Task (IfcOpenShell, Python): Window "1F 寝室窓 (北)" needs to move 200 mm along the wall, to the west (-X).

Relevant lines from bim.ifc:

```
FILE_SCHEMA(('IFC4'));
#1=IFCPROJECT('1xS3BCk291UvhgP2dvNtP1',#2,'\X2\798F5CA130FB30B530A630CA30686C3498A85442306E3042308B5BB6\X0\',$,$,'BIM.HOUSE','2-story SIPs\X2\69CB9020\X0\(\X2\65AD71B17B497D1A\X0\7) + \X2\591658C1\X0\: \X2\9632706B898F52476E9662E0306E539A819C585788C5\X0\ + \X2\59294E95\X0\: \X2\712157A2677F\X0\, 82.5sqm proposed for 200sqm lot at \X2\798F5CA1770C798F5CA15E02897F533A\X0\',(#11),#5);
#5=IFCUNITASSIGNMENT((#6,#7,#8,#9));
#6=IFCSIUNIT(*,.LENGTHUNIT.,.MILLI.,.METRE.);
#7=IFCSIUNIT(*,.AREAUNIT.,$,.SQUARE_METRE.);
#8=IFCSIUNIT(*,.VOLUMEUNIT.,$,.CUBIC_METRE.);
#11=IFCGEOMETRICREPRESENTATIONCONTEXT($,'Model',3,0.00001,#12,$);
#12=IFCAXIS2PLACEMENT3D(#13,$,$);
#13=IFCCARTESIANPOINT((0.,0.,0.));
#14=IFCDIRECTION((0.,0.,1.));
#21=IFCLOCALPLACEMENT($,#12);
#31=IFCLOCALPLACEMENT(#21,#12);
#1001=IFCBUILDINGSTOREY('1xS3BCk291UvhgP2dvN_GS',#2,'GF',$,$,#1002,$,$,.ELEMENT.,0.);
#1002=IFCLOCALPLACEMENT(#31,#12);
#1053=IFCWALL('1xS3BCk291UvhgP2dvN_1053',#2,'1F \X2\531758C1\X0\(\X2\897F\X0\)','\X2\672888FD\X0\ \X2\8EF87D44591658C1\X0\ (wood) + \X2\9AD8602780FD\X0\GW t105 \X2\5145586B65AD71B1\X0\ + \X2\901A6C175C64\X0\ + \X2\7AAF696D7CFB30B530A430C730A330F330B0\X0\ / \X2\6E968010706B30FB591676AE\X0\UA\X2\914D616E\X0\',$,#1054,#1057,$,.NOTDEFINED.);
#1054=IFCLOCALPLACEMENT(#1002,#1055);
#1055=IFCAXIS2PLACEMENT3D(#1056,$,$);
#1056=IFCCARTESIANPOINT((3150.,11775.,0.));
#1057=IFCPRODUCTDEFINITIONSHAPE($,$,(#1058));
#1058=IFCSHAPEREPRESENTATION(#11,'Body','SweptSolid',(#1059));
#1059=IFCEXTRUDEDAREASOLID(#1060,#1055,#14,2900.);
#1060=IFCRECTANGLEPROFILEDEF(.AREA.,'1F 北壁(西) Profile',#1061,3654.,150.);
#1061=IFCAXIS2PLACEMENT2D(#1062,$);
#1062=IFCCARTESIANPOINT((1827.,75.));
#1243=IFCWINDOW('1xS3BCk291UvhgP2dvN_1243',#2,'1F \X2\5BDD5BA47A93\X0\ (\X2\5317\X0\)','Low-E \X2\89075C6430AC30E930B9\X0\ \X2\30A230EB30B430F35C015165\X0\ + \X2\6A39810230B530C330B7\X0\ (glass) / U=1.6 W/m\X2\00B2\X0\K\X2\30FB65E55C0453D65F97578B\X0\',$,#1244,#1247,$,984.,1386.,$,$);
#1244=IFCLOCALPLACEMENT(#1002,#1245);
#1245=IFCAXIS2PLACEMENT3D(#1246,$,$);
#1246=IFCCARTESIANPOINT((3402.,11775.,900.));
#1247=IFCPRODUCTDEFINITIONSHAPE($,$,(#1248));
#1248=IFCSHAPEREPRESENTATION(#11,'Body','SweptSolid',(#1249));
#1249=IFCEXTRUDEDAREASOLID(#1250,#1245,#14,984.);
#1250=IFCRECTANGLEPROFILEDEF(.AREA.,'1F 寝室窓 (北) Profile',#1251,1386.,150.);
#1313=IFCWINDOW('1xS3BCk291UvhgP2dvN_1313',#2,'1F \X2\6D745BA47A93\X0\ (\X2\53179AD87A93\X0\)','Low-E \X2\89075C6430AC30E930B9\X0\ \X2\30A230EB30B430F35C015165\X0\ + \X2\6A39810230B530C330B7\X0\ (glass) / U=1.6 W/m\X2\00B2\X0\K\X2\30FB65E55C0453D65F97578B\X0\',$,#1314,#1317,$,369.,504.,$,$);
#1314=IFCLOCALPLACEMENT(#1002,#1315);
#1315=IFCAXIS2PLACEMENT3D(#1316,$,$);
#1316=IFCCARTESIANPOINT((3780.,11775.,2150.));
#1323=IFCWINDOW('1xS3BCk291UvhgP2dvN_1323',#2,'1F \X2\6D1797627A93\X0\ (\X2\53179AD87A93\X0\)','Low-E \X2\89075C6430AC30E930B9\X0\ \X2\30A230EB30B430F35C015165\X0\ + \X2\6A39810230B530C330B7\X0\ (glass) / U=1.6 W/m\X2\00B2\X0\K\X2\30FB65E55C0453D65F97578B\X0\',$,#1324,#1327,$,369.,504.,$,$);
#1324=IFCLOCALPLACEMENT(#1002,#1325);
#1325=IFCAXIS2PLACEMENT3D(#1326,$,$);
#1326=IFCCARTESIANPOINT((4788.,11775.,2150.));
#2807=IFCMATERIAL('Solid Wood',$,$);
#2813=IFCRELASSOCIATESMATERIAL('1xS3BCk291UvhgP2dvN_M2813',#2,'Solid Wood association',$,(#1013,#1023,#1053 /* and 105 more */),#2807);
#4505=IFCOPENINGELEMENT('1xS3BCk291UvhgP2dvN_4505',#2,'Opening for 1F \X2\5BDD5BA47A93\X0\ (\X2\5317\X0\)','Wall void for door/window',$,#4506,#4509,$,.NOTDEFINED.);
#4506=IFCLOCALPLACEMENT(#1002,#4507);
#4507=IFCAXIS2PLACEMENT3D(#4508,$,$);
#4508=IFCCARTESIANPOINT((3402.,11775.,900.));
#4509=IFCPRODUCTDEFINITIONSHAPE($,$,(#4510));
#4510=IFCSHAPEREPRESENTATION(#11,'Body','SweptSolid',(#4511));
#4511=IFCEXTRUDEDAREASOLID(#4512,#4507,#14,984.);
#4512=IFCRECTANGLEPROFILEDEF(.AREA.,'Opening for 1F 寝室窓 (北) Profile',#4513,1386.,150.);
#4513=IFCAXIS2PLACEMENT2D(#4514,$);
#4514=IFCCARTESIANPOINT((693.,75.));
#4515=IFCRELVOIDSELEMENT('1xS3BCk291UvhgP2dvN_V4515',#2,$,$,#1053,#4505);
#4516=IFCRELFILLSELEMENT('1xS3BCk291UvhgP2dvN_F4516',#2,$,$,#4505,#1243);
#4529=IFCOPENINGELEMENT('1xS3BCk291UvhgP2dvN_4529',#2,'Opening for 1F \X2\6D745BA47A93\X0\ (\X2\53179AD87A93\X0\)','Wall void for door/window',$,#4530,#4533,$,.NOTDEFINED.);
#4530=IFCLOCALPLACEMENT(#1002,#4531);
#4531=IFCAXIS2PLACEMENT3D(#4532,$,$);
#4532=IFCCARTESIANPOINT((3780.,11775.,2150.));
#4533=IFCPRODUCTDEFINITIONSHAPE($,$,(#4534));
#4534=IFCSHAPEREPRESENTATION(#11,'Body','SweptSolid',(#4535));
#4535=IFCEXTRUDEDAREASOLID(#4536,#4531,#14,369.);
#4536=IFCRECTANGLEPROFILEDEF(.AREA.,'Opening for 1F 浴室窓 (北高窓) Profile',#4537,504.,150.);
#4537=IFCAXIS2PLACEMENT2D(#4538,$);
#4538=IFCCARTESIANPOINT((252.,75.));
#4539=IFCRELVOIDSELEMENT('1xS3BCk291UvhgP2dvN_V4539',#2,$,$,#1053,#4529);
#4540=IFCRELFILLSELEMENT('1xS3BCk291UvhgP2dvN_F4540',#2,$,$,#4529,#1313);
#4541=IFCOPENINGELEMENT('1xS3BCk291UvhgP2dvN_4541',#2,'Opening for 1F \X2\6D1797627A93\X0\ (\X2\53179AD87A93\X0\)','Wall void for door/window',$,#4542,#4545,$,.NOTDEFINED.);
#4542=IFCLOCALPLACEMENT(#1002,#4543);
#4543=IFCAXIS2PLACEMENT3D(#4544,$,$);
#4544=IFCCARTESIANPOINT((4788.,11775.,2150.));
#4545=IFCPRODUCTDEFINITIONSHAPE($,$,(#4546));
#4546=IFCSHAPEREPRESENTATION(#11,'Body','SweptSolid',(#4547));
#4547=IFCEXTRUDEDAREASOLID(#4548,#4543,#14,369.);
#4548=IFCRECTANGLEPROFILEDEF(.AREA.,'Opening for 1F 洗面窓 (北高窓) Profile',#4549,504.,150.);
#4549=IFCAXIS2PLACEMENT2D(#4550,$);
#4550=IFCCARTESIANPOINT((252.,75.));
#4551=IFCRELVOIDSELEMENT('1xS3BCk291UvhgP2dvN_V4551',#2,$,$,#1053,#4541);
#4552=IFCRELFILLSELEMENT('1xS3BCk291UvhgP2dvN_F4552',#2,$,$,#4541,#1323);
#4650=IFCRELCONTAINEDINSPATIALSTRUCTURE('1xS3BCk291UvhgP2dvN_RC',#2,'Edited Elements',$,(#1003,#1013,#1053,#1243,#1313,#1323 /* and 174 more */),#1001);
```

```python
import ifcopenshell
import ifcopenshell.api.geometry
import ifcopenshell.util.placement

model = ifcopenshell.open("bim.ifc")

window = model.by_guid("1xS3BCk291UvhgP2dvN_1243")
opening = window.FillsVoids[0].RelatingOpeningElement
wall = opening.VoidsElements[0].RelatingBuildingElement

wall_matrix = ifcopenshell.util.placement.get_local_placement(wall.ObjectPlacement)
shift = wall_matrix[:3, 0] * -200.0
before = ifcopenshell.util.placement.get_local_placement(window.ObjectPlacement)[:3, 3].copy()

# The window is not placed relative to its opening, so move both.
for product in (opening, window):
    matrix = ifcopenshell.util.placement.get_local_placement(product.ObjectPlacement)
    matrix[:3, 3] += shift
    ifcopenshell.api.geometry.edit_object_placement(model, product=product, matrix=matrix, is_si=False)

after = ifcopenshell.util.placement.get_local_placement(window.ObjectPlacement)[:3, 3]
print("window moved by", (after - before).round(3) + 0.0)

model.write("bim_edited.ifc")
```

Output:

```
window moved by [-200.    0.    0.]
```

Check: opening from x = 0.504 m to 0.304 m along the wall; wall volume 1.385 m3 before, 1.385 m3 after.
